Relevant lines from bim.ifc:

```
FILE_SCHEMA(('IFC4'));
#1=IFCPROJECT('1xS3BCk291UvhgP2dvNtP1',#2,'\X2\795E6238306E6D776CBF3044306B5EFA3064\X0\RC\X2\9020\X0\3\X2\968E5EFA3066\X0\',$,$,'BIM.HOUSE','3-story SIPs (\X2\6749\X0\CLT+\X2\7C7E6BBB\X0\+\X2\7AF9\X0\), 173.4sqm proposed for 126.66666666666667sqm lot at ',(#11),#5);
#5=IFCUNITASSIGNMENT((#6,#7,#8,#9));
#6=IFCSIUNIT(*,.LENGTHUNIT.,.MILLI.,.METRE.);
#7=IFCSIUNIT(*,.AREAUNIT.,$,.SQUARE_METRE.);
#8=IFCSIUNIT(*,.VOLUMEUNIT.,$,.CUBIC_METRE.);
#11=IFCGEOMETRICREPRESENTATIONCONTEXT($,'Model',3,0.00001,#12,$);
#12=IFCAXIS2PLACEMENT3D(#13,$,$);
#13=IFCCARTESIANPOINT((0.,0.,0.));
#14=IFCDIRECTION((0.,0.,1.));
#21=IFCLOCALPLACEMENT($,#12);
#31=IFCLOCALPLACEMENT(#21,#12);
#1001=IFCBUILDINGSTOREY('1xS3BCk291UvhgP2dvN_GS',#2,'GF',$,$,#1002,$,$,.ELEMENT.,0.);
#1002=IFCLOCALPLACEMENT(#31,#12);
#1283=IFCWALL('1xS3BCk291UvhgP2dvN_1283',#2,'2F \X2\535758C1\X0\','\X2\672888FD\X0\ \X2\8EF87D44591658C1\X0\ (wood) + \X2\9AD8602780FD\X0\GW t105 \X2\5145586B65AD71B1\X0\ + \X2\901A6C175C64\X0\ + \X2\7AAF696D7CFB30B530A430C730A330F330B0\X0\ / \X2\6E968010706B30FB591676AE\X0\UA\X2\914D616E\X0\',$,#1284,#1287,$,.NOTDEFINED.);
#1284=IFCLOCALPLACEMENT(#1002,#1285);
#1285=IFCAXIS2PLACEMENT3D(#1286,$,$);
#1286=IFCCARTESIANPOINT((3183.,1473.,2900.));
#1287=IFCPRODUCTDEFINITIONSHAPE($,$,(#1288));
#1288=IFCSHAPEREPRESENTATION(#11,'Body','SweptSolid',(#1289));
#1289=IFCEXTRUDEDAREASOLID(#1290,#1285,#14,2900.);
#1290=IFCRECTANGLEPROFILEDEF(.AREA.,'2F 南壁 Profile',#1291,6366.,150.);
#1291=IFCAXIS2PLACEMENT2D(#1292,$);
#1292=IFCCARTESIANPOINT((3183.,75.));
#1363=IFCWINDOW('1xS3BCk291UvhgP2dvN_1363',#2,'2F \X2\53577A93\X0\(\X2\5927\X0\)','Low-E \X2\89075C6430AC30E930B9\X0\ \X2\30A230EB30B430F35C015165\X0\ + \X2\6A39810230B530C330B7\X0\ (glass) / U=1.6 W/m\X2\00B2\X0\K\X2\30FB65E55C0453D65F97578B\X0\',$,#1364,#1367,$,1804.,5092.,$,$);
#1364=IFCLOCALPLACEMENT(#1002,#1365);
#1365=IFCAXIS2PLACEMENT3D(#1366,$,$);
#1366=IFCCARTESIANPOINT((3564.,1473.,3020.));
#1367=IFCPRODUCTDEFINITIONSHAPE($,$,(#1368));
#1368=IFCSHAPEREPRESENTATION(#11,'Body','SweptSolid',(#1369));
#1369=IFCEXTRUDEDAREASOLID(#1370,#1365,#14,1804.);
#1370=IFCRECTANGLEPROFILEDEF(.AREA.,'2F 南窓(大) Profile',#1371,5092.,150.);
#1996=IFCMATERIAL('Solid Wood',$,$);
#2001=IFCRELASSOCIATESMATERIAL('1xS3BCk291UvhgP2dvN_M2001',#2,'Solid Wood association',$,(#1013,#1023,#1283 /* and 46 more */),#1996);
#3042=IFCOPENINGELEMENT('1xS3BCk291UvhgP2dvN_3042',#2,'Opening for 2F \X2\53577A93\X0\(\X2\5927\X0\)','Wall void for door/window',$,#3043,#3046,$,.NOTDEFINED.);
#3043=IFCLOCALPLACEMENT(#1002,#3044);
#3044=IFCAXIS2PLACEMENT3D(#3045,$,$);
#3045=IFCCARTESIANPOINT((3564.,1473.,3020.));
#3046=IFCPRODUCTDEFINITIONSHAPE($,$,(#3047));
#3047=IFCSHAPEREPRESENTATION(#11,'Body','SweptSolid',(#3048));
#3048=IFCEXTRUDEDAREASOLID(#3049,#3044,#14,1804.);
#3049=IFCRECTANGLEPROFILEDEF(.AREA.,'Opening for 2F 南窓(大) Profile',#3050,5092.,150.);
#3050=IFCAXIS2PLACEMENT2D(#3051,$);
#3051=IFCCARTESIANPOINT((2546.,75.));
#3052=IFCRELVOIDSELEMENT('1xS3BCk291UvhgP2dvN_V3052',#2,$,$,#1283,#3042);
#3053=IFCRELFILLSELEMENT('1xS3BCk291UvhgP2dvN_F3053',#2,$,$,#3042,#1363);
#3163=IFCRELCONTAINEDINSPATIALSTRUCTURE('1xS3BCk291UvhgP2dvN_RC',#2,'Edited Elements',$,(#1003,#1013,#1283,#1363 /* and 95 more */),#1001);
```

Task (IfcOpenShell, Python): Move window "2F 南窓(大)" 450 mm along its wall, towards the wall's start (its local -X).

```python
import ifcopenshell
import ifcopenshell.api.geometry
import ifcopenshell.util.placement
import ifcopenshell.util.unit

model = ifcopenshell.open("bim.ifc")
unit_scale = ifcopenshell.util.unit.calculate_unit_scale(model)

window = model.by_guid("1xS3BCk291UvhgP2dvN_1363")
opening = window.FillsVoids[0].RelatingOpeningElement
wall = opening.VoidsElements[0].RelatingBuildingElement

wall_matrix = ifcopenshell.util.placement.get_local_placement(wall.ObjectPlacement)
shift = wall_matrix[:3, 0] * -0.45 / unit_scale
before = ifcopenshell.util.placement.get_local_placement(window.ObjectPlacement)[:3, 3].copy()

# The window is not placed relative to its opening, so move both.
for product in (opening, window):
    matrix = ifcopenshell.util.placement.get_local_placement(product.ObjectPlacement)
    matrix[:3, 3] += shift
    ifcopenshell.api.geometry.edit_object_placement(model, product=product, matrix=matrix, is_si=False)

after = ifcopenshell.util.placement.get_local_placement(window.ObjectPlacement)[:3, 3]
print("window moved by", (after - before).round(3) + 0.0)

model.write("bim_v2.ifc")
```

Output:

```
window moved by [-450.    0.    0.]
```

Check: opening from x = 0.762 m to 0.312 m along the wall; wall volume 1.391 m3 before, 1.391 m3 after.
